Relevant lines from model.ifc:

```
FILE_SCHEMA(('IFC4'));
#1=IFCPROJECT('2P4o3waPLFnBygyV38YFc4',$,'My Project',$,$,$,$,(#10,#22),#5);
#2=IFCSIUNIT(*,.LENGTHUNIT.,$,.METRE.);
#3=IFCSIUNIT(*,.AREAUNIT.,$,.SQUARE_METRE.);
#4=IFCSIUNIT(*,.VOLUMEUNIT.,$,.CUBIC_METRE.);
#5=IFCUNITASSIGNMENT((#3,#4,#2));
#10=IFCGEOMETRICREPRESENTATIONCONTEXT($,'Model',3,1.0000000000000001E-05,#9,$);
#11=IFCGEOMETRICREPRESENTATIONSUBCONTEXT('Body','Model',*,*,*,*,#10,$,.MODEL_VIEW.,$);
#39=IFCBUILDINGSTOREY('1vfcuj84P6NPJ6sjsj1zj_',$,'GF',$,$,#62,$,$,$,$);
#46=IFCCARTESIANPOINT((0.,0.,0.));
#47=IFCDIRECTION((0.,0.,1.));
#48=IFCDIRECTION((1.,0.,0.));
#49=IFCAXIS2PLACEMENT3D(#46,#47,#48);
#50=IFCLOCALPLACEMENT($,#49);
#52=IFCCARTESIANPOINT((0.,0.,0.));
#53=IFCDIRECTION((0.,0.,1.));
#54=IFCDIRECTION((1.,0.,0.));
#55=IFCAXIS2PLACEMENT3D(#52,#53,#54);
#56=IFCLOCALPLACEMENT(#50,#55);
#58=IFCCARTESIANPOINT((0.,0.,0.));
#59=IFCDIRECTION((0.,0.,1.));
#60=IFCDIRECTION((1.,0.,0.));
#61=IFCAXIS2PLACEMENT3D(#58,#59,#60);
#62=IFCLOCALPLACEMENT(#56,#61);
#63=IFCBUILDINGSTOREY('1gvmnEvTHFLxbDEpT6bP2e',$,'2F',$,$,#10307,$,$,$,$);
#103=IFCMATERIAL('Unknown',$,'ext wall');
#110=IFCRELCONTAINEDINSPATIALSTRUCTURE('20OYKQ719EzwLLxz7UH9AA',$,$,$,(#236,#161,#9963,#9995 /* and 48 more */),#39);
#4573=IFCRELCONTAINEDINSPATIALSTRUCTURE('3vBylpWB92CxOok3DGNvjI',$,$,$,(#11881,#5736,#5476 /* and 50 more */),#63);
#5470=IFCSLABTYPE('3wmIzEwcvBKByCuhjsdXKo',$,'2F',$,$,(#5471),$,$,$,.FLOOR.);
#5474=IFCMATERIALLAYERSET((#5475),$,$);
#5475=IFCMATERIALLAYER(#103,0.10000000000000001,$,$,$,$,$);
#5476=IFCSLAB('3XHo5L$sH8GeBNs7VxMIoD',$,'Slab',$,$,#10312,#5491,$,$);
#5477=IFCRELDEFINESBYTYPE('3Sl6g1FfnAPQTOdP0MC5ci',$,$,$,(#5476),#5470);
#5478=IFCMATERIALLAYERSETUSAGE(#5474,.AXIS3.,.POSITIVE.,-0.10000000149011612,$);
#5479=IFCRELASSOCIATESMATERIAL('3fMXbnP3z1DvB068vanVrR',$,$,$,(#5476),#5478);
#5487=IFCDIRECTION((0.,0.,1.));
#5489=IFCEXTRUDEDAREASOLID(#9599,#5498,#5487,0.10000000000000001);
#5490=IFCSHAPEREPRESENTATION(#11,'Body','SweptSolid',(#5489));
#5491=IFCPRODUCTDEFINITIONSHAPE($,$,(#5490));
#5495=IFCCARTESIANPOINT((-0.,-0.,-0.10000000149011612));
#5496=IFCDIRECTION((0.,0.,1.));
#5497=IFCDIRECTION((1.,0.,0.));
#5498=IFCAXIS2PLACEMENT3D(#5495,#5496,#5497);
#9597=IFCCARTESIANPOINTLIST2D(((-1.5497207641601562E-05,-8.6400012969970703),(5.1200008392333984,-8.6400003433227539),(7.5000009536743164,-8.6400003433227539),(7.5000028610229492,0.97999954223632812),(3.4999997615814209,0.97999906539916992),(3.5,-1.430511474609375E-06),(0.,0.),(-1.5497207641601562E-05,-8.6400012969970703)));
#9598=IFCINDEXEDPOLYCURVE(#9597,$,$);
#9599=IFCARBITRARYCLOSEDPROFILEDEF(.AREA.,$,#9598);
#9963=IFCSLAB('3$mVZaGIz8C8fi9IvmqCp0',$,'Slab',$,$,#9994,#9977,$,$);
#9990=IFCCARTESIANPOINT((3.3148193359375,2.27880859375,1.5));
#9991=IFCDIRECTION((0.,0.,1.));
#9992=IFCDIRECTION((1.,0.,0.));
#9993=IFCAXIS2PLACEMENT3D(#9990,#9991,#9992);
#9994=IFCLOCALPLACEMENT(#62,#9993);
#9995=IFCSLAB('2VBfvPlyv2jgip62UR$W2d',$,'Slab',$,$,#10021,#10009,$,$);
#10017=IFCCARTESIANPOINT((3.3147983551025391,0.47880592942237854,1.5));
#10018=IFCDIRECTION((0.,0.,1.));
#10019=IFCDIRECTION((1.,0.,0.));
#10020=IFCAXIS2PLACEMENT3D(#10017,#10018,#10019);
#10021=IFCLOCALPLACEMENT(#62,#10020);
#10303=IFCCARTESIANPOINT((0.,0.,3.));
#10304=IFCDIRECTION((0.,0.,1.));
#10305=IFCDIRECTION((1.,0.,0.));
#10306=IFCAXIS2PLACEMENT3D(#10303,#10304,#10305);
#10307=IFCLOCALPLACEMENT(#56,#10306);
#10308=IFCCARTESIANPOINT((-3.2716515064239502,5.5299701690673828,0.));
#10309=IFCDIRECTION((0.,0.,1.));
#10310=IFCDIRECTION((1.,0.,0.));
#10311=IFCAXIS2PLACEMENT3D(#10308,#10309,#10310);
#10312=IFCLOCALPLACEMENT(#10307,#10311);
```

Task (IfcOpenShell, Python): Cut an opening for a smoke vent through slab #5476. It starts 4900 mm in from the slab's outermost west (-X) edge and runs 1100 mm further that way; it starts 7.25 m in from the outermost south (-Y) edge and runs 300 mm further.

```python
import numpy as np
import ifcopenshell
import ifcopenshell.api.feature
import ifcopenshell.api.geometry
import ifcopenshell.api.root
import ifcopenshell.geom
import ifcopenshell.util.placement
import ifcopenshell.util.representation
import ifcopenshell.util.shape
import ifcopenshell.util.unit

model = ifcopenshell.open("model.ifc")
unit_scale = ifcopenshell.util.unit.calculate_unit_scale(model)
settings = ifcopenshell.geom.settings()


def volume(element):
    """Net volume in cubic metres, openings subtracted."""
    shape = ifcopenshell.geom.create_shape(settings, element)
    return ifcopenshell.util.shape.get_volume(shape.geometry)


slab = model.by_guid("3XHo5L$sH8GeBNs7VxMIoD")
before = volume(slab)

# Extent in the slab's own axes, in metres. The edges named are its -X and -Y sides.
slab_shape = ifcopenshell.geom.create_shape(settings, slab)
vertices = ifcopenshell.util.shape.get_vertices(slab_shape.geometry)
x_min, y_min, bottom = vertices.min(axis=0)
top = vertices[:, 2].max()

opening = ifcopenshell.api.root.create_entity(model, ifc_class="IfcOpeningElement", name="Smoke vent opening", predefined_type="OPENING")
context = ifcopenshell.util.representation.get_context(model, "Model", "Body", "MODEL_VIEW")
width, depth = 1.1, 0.3
outline = [(0.0, 0.0), (width, 0.0), (width, depth), (0.0, depth), (0.0, 0.0)]
# Overshoot both faces by 50 mm so the cut is clean.
shape = ifcopenshell.api.geometry.add_slab_representation(
    model, context=context, depth=top - bottom + 0.1, polyline=outline
)
ifcopenshell.api.geometry.assign_representation(model, product=opening, representation=shape)

matrix = ifcopenshell.util.placement.get_local_placement(slab.ObjectPlacement)
matrix[:, 3] = matrix @ np.append(np.array([x_min + 4.9, y_min + 7.25, bottom - 0.05]) / unit_scale, 1.0)
ifcopenshell.api.geometry.edit_object_placement(model, product=opening, matrix=matrix, is_si=False)
ifcopenshell.api.feature.add_feature(model, feature=opening, element=slab)

after = volume(slab)

print(f"slab volume {before:.3f} -> {after:.3f} m3")

model.write("model_v2.ifc")
```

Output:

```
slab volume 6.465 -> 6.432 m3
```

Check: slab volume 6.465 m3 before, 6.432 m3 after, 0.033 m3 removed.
